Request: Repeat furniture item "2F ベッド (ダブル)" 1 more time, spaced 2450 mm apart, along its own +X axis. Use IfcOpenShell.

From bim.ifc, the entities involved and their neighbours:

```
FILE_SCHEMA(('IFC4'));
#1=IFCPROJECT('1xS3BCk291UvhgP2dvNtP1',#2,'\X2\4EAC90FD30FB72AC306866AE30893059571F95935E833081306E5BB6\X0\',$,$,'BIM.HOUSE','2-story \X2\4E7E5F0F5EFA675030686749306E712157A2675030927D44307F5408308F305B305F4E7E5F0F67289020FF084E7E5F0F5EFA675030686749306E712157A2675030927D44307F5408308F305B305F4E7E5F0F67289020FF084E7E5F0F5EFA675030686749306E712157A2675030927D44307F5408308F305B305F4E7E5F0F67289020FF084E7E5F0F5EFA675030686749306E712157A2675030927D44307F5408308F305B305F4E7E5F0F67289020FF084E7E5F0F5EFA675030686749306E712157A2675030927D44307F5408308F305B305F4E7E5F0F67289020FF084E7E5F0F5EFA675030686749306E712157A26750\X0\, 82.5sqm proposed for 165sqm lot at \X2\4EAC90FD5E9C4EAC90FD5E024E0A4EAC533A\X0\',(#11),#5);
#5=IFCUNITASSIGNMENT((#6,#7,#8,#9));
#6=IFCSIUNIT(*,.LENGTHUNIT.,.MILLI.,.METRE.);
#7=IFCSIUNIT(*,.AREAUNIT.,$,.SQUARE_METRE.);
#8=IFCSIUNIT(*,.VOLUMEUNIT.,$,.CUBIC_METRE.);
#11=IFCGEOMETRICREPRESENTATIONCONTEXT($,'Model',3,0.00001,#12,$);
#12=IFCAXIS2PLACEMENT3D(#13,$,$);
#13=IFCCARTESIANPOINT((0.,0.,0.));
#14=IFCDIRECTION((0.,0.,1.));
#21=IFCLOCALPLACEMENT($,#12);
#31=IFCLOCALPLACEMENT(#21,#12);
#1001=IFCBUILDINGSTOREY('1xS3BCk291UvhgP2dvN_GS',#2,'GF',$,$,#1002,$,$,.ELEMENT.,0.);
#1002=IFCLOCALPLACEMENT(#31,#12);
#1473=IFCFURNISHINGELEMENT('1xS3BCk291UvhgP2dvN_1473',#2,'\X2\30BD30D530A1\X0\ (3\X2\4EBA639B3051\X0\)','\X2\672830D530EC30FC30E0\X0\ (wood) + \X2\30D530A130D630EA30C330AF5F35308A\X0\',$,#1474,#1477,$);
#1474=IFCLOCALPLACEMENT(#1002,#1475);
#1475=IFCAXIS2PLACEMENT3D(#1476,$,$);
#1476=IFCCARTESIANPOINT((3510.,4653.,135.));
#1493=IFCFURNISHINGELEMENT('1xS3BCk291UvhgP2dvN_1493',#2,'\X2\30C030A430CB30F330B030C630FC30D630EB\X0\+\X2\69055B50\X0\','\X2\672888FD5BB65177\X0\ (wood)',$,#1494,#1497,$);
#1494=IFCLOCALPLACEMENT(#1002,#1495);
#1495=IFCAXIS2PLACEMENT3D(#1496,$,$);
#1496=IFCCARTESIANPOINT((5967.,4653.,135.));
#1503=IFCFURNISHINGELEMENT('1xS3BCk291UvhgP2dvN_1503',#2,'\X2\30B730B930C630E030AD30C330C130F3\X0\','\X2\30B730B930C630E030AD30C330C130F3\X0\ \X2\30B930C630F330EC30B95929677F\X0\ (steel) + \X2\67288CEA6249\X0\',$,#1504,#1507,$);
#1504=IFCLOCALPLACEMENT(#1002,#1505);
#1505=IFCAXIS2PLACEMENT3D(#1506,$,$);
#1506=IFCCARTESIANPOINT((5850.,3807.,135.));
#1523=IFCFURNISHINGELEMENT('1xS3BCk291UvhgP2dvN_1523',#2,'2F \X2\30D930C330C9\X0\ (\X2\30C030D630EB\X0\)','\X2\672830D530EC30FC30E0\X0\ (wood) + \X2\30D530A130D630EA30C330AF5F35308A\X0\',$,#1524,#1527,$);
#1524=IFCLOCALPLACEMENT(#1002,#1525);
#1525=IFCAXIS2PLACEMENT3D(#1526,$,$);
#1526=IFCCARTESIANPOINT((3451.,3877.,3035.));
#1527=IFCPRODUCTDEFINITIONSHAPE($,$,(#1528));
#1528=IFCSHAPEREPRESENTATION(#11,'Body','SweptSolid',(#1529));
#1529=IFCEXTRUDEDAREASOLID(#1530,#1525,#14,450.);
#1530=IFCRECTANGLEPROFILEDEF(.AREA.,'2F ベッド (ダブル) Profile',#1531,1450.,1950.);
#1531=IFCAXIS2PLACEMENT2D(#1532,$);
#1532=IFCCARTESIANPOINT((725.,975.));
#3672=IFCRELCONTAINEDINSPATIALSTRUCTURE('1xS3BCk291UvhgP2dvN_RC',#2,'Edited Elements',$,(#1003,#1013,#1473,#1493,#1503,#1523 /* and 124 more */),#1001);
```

```python
import ifcopenshell
import ifcopenshell.api.geometry
import ifcopenshell.api.root
import ifcopenshell.util.element
import ifcopenshell.util.placement
import ifcopenshell.util.unit

model = ifcopenshell.open("bim.ifc")
unit_scale = ifcopenshell.util.unit.calculate_unit_scale(model)


def reuse_history(source, copy):
    """copy_class also copies each property set's owner history, people and application; keep the originals."""
    for rel in copy.IsDefinedBy:
        if rel.is_a("IfcRelDefinesByProperties") and (history := rel.RelatingPropertyDefinition.OwnerHistory):
            rel.RelatingPropertyDefinition.OwnerHistory = source.OwnerHistory
            ifcopenshell.util.element.remove_deep2(model, history)


source = model.by_id(1523)
base = ifcopenshell.util.placement.get_local_placement(source.ObjectPlacement)
step = base[:3, 0] * 2.45 / unit_scale

for i in range(1, 2):
    copy = ifcopenshell.api.root.copy_class(model, product=source)
    copy.Representation = ifcopenshell.util.element.copy_deep(
        model, source.Representation, exclude=["IfcGeometricRepresentationContext", "IfcRepresentationMap"]
    )
    reuse_history(source, copy)
    matrix = base.copy()
    matrix[:3, 3] += i * step
    print("added at", matrix[:3, 3].round(3) + 0.0)
    ifcopenshell.api.geometry.edit_object_placement(model, product=copy, matrix=matrix, is_si=False)

model.write("bim-out.ifc")
```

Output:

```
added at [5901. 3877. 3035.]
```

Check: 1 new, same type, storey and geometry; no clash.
